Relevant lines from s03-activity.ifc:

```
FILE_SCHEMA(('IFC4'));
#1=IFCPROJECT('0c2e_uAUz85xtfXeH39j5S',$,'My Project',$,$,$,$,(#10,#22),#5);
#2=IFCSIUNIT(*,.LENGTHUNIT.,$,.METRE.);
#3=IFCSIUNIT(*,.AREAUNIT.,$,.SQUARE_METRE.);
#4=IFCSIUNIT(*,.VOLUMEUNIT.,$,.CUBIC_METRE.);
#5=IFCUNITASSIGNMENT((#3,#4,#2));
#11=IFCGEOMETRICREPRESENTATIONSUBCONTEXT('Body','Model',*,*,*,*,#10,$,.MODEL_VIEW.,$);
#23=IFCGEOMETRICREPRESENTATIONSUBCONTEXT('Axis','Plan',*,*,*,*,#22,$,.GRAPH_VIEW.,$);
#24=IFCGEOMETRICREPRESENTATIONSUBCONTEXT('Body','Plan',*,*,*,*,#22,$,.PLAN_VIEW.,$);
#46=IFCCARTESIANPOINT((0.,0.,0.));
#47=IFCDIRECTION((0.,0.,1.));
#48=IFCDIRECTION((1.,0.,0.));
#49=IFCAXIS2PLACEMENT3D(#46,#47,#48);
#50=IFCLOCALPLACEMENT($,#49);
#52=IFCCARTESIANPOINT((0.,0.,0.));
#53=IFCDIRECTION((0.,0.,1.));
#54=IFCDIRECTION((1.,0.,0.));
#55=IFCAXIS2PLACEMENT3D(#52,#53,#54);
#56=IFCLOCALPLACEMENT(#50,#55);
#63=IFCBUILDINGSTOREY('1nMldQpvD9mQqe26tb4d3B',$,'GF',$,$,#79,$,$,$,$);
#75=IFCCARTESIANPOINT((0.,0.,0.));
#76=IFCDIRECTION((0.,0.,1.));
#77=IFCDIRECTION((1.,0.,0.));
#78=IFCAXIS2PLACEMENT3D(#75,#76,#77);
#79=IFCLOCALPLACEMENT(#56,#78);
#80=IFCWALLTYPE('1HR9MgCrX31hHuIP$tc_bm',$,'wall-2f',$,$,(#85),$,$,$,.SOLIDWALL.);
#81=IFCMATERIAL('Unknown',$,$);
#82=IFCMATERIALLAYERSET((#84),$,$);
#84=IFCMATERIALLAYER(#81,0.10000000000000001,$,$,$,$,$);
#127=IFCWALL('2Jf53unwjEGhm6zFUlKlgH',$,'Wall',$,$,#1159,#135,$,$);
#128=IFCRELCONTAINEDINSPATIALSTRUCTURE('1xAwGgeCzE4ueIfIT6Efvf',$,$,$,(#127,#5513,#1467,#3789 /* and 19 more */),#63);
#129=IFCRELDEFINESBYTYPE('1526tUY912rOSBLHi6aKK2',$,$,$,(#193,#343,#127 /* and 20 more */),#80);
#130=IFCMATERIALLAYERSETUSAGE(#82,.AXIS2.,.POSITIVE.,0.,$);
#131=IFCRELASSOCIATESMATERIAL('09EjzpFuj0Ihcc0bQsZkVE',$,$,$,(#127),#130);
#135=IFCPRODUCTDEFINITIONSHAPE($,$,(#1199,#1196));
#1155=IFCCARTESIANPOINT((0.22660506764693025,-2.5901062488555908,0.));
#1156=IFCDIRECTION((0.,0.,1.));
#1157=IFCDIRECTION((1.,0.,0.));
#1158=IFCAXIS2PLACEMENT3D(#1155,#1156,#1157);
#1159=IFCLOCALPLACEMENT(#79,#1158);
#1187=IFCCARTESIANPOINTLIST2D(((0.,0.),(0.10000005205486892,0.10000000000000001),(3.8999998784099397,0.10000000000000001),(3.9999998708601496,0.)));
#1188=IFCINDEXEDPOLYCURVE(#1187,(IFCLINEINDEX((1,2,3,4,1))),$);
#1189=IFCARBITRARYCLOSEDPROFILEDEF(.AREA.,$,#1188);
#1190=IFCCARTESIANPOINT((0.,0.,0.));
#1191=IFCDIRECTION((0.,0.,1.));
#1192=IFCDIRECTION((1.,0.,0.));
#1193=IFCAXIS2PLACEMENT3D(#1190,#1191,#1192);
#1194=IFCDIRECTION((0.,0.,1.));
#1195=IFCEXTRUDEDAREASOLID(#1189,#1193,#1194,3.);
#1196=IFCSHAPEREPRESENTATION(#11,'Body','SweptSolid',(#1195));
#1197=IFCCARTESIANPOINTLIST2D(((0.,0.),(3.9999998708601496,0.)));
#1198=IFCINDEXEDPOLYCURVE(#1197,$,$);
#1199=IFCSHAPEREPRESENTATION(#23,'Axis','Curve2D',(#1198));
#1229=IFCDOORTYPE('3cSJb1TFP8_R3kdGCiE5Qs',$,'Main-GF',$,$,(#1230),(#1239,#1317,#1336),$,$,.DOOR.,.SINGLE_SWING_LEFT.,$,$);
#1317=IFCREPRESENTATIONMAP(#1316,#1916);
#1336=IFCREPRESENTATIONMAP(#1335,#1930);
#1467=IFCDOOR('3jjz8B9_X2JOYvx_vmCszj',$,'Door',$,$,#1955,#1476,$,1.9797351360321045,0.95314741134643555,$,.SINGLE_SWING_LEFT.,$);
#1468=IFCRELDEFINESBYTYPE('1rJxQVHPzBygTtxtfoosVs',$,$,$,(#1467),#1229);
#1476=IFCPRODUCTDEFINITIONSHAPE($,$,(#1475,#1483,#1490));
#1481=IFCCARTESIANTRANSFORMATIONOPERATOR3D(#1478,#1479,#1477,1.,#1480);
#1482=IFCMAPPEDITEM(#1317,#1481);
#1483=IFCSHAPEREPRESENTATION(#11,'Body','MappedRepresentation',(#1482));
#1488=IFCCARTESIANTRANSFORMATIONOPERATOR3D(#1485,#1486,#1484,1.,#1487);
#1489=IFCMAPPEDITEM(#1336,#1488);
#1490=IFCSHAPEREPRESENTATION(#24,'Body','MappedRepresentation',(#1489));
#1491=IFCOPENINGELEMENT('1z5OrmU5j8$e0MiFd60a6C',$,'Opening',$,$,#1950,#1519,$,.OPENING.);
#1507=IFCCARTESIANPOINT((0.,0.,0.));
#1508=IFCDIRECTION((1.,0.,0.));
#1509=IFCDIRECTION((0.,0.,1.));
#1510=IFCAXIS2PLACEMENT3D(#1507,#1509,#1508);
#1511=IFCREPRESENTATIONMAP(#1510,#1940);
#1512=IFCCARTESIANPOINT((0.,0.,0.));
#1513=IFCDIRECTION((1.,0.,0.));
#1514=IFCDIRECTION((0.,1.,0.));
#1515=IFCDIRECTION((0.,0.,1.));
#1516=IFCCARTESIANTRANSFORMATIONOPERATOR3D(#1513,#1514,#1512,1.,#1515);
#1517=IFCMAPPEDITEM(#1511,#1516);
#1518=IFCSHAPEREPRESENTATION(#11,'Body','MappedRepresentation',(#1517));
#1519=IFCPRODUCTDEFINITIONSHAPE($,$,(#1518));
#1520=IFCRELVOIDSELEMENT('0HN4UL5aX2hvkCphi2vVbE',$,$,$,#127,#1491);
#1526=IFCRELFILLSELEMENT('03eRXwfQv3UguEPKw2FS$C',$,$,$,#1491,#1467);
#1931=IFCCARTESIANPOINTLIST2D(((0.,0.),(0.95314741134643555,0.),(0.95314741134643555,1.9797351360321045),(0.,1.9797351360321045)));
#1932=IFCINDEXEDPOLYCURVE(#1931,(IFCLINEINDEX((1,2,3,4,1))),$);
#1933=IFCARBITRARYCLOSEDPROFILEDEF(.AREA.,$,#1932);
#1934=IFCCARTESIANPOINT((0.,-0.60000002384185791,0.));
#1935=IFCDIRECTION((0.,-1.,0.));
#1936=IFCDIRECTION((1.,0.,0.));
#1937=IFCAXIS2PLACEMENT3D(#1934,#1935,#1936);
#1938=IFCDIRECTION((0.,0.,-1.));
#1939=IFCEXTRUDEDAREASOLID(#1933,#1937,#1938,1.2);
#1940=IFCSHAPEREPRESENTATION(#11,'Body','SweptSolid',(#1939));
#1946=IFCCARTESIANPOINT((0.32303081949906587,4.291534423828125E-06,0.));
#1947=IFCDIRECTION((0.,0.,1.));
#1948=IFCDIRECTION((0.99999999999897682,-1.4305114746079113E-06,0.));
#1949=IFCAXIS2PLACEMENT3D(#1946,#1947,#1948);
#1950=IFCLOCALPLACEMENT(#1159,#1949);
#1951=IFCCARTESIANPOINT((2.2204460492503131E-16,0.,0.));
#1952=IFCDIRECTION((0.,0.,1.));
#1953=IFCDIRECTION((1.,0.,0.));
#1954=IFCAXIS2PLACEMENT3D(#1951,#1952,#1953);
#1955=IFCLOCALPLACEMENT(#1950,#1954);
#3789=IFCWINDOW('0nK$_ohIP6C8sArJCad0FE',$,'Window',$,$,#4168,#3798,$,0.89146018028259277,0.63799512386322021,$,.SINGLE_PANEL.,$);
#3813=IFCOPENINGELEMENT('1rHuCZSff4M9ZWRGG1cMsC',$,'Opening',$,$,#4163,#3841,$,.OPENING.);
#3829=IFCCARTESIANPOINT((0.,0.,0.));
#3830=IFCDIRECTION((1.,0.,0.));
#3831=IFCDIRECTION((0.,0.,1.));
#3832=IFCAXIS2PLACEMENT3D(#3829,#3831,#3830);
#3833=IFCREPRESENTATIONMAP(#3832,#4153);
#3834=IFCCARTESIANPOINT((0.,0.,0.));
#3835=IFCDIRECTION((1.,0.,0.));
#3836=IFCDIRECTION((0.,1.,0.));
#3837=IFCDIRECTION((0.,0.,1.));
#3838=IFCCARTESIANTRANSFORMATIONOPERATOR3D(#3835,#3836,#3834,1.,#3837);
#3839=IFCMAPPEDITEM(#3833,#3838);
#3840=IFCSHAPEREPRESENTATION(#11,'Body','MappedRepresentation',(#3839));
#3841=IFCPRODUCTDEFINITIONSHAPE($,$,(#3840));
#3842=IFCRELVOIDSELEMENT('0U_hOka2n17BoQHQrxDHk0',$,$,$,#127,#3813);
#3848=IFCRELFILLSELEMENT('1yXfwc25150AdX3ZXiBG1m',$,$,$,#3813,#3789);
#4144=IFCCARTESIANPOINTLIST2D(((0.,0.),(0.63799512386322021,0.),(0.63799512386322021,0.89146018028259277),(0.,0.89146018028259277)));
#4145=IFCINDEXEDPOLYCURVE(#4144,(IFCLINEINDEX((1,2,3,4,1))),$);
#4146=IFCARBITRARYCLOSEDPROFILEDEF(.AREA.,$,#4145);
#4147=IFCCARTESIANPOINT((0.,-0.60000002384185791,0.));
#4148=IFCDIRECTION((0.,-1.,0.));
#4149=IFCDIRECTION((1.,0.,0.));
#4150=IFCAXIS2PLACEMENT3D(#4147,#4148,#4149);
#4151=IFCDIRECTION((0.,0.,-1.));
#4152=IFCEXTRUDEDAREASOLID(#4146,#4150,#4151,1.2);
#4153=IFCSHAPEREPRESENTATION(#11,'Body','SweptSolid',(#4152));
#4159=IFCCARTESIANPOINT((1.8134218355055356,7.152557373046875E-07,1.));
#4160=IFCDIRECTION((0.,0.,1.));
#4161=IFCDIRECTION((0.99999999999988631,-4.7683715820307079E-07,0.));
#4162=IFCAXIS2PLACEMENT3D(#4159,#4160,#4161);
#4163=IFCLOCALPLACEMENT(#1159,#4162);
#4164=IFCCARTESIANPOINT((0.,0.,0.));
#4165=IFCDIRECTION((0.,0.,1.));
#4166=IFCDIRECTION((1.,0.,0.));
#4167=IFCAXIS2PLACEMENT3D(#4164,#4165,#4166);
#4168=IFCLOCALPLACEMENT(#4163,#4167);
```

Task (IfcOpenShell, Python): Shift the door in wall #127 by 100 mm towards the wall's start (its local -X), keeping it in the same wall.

```python
import ifcopenshell
import ifcopenshell.api.geometry
import ifcopenshell.util.placement
import ifcopenshell.util.unit

model = ifcopenshell.open("s03-activity.ifc")
unit_scale = ifcopenshell.util.unit.calculate_unit_scale(model)

door = model.by_id(1467)
opening = door.FillsVoids[0].RelatingOpeningElement
wall = opening.VoidsElements[0].RelatingBuildingElement

wall_matrix = ifcopenshell.util.placement.get_local_placement(wall.ObjectPlacement)
shift = wall_matrix[:3, 0] * -0.1 / unit_scale
before = ifcopenshell.util.placement.get_local_placement(door.ObjectPlacement)[:3, 3].copy()

# The door is placed relative to its opening, so it follows when the opening moves.
matrix = ifcopenshell.util.placement.get_local_placement(opening.ObjectPlacement)
matrix[:3, 3] += shift
ifcopenshell.api.geometry.edit_object_placement(
    model, product=opening, matrix=matrix, is_si=False, should_transform_children=True
)

after = ifcopenshell.util.placement.get_local_placement(door.ObjectPlacement)[:3, 3]
print("door moved by", (after - before).round(3) + 0.0)

model.write("s03-activity_v2.ifc")
```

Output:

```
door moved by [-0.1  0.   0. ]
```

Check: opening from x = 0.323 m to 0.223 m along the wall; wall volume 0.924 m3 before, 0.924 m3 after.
